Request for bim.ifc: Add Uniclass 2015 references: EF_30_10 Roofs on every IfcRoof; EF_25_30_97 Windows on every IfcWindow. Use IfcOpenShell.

First a look at what the model holds.

```python
import ifcopenshell

model = ifcopenshell.open("bim.ifc")
print(model.schema)
print("classifications:", [c.Name for c in model.by_type("IfcClassification")])
for ifc_class in ("IfcDoor", "IfcRoof", "IfcStair", "IfcWall", "IfcWindow"):
    print(ifc_class, len(model.by_type(ifc_class)))
```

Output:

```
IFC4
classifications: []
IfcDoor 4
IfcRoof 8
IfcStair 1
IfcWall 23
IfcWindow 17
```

```python
import ifcopenshell
import ifcopenshell.api.classification

model = ifcopenshell.open("bim.ifc")

system = ifcopenshell.api.classification.add_classification(model, classification="Uniclass 2015")

codes = {
    "IfcRoof": ("EF_30_10", "Roofs"),
    "IfcWindow": ("EF_25_30_97", "Windows"),
}
for ifc_class, (code, name) in codes.items():
    products = model.by_type(ifc_class)
    ifcopenshell.api.classification.add_reference(
        model, products=products, classification=system, identification=code, name=name
    )
    print(code, len(products))

model.write("bim_updated.ifc")
```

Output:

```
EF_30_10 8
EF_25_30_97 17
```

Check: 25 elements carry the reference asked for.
